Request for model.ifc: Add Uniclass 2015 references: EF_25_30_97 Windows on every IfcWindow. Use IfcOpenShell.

First a look at what the model holds.

```python
import ifcopenshell

model = ifcopenshell.open("model.ifc")
print(model.schema)
print("classifications:", [c.Name for c in model.by_type("IfcClassification")])
for ifc_class in ("IfcDoor", "IfcRoof", "IfcStair", "IfcWall", "IfcWindow"):
    print(ifc_class, len(model.by_type(ifc_class)))
```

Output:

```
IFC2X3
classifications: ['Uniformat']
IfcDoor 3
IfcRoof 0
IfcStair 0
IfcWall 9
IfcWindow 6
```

```python
import ifcopenshell
import ifcopenshell.api.classification

model = ifcopenshell.open("model.ifc")

# IFC2X3 requires Source and Edition and has no link from the project to the system.
system = model.create_entity("IfcClassification", Source="NBS", Edition="2015", Name="Uniclass 2015")

codes = {
    "IfcWindow": ("EF_25_30_97", "Windows"),
}
for ifc_class, (code, name) in codes.items():
    products = model.by_type(ifc_class)
    ifcopenshell.api.classification.add_reference(
        model, products=products, classification=system, identification=code, name=name
    )
    print(code, len(products))

model.write("model_edited.ifc")
```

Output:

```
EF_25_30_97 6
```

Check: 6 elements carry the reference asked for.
